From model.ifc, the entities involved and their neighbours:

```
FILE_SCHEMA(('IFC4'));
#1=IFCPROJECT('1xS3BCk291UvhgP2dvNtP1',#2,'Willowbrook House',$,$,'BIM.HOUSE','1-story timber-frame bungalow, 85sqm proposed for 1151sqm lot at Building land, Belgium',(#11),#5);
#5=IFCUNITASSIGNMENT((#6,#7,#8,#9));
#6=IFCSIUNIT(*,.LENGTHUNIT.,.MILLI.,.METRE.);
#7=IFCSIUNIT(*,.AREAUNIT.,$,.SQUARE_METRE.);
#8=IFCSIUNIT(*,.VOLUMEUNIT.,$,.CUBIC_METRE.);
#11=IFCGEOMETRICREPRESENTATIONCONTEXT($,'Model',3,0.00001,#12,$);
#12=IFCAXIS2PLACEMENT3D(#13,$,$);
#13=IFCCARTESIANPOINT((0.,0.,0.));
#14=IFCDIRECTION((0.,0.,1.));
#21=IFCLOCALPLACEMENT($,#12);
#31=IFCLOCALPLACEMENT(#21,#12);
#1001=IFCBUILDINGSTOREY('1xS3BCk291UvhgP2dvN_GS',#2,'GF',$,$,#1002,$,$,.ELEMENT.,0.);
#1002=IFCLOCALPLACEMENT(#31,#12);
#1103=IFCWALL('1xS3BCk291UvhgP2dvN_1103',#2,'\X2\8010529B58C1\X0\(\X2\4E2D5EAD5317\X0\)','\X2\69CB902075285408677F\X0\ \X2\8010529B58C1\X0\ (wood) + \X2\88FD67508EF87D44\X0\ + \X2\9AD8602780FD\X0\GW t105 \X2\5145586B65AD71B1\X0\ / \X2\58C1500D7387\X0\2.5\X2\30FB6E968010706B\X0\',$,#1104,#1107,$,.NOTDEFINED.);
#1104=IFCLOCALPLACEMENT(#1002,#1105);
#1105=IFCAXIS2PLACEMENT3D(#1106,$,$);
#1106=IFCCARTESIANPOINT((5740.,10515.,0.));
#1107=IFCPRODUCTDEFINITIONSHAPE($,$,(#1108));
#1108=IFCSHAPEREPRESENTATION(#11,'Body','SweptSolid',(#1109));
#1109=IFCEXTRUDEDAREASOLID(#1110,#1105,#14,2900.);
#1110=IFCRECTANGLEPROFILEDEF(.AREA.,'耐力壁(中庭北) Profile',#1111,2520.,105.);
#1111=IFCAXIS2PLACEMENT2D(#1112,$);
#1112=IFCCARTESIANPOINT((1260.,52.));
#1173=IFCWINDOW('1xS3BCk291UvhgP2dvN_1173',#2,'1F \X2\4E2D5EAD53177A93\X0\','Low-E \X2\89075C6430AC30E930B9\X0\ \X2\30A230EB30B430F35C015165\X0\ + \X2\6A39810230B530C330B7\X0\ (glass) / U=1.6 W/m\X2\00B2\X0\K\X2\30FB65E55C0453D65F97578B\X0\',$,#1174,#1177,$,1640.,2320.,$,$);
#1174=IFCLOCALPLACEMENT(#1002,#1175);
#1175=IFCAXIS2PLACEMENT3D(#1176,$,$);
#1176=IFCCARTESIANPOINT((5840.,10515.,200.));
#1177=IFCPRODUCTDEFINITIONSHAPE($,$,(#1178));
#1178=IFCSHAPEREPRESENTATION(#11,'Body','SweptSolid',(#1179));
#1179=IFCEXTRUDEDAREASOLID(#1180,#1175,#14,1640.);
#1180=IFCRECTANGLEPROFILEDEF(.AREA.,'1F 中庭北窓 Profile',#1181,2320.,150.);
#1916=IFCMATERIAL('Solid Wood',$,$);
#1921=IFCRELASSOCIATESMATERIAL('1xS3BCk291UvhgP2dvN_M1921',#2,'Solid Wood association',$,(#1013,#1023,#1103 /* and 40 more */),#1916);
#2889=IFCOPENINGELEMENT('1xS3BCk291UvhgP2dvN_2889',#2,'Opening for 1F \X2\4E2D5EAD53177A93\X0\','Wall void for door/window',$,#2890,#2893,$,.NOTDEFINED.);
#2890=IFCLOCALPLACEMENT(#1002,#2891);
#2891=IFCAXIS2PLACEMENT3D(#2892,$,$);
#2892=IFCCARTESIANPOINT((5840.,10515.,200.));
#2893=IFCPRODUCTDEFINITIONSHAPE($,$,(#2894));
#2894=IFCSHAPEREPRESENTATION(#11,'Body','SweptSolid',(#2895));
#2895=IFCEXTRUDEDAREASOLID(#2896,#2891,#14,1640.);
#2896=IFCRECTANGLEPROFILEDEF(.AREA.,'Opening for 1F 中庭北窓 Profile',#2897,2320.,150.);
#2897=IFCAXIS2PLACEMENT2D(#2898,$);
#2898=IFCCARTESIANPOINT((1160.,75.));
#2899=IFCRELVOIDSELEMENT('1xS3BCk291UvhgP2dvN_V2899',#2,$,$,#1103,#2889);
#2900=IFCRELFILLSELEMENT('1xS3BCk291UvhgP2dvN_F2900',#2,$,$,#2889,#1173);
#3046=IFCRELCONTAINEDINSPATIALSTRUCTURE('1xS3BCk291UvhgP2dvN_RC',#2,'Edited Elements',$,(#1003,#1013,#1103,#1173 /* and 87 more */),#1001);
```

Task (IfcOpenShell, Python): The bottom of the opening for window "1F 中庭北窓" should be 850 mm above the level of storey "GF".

```python
import numpy as np
import ifcopenshell
import ifcopenshell.api.geometry
import ifcopenshell.geom
import ifcopenshell.util.element
import ifcopenshell.util.placement
import ifcopenshell.util.shape
import ifcopenshell.util.unit

model = ifcopenshell.open("model.ifc")
unit_scale = ifcopenshell.util.unit.calculate_unit_scale(model)

window = model.by_guid("1xS3BCk291UvhgP2dvN_1173")
opening = window.FillsVoids[0].RelatingOpeningElement
storey = ifcopenshell.util.element.get_container(window, ifc_class="IfcBuildingStorey")
level = ifcopenshell.util.placement.get_local_placement(storey.ObjectPlacement)[2, 3]

# The opening's origin need not be at the sill, so measure its lowest point.
shape = ifcopenshell.geom.create_shape(ifcopenshell.geom.settings(), opening)
bottom = ifcopenshell.util.shape.get_shape_bottom_elevation(shape, shape.geometry) / unit_scale
dz = level + 850.0 - bottom

shift = np.array([0.0, 0.0, dz])
# The window is not placed relative to its opening, so move both.
for product in (opening, window):
    matrix = ifcopenshell.util.placement.get_local_placement(product.ObjectPlacement)
    matrix[:3, 3] += shift
    ifcopenshell.api.geometry.edit_object_placement(model, product=product, matrix=matrix, is_si=False)

print(f"moved by {dz * unit_scale:+.3f} m")

model.write("model_updated.ifc")
```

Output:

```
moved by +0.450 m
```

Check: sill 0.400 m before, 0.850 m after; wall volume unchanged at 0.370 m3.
